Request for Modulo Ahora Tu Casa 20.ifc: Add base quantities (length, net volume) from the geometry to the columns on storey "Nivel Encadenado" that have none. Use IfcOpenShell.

First a look at what the model holds.

```python
import ifcopenshell
import ifcopenshell.util.element
import ifcopenshell.util.unit

model = ifcopenshell.open("Modulo Ahora Tu Casa 20.ifc")
print(model.schema)
for unit_type in ("LENGTHUNIT", "AREAUNIT", "VOLUMEUNIT"):
    print(unit_type, ifcopenshell.util.unit.calculate_unit_scale(model, unit_type))
storey = next(s for s in model.by_type("IfcBuildingStorey") if s.Name == "Nivel Encadenado")
columns = [e for e in ifcopenshell.util.element.get_decomposition(storey) if e.is_a("IfcColumn")]
for e in sorted(columns, key=lambda e: e.id()):
    print(e.id(), e.is_a(), e.Name, list(ifcopenshell.util.element.get_psets(e, qtos_only=True)), sep=" | ")
```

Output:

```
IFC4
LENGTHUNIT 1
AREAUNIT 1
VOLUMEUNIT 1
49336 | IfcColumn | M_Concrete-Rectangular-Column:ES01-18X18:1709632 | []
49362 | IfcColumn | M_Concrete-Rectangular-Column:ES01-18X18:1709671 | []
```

```python
import ifcopenshell
import ifcopenshell.api.pset
import ifcopenshell.geom
import ifcopenshell.util.element
import ifcopenshell.util.shape
import ifcopenshell.util.unit

model = ifcopenshell.open("Modulo Ahora Tu Casa 20.ifc")
unit_scale = ifcopenshell.util.unit.calculate_unit_scale(model)
volume_scale = ifcopenshell.util.unit.calculate_unit_scale(model, "VOLUMEUNIT")
settings = ifcopenshell.geom.settings()

storey = next(s for s in model.by_type("IfcBuildingStorey") if s.Name == "Nivel Encadenado")
columns = [e for e in ifcopenshell.util.element.get_decomposition(storey) if e.is_a("IfcColumn")]

for e in sorted(columns, key=lambda e: e.id()):
    if ifcopenshell.util.element.get_psets(e, qtos_only=True, should_inherit=False):
        continue
    # Geometry comes back in metres, in the element's own axes.
    shape = ifcopenshell.geom.create_shape(settings, e)
    values = {
        "Length": ifcopenshell.util.shape.get_z(shape.geometry) / unit_scale,
        "NetVolume": ifcopenshell.util.shape.get_volume(shape.geometry) / volume_scale,
    }
    qto = ifcopenshell.api.pset.add_qto(model, product=e, name="Qto_ColumnBaseQuantities")
    ifcopenshell.api.pset.edit_qto(model, qto=qto, properties=values)
    print(e.id(), {k: round(v, 3) for k, v in values.items()})

model.write("Modulo Ahora Tu Casa 20_edited.ifc")
```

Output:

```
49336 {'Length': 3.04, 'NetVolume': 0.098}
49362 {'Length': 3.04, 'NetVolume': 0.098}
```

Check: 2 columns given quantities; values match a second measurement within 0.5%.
